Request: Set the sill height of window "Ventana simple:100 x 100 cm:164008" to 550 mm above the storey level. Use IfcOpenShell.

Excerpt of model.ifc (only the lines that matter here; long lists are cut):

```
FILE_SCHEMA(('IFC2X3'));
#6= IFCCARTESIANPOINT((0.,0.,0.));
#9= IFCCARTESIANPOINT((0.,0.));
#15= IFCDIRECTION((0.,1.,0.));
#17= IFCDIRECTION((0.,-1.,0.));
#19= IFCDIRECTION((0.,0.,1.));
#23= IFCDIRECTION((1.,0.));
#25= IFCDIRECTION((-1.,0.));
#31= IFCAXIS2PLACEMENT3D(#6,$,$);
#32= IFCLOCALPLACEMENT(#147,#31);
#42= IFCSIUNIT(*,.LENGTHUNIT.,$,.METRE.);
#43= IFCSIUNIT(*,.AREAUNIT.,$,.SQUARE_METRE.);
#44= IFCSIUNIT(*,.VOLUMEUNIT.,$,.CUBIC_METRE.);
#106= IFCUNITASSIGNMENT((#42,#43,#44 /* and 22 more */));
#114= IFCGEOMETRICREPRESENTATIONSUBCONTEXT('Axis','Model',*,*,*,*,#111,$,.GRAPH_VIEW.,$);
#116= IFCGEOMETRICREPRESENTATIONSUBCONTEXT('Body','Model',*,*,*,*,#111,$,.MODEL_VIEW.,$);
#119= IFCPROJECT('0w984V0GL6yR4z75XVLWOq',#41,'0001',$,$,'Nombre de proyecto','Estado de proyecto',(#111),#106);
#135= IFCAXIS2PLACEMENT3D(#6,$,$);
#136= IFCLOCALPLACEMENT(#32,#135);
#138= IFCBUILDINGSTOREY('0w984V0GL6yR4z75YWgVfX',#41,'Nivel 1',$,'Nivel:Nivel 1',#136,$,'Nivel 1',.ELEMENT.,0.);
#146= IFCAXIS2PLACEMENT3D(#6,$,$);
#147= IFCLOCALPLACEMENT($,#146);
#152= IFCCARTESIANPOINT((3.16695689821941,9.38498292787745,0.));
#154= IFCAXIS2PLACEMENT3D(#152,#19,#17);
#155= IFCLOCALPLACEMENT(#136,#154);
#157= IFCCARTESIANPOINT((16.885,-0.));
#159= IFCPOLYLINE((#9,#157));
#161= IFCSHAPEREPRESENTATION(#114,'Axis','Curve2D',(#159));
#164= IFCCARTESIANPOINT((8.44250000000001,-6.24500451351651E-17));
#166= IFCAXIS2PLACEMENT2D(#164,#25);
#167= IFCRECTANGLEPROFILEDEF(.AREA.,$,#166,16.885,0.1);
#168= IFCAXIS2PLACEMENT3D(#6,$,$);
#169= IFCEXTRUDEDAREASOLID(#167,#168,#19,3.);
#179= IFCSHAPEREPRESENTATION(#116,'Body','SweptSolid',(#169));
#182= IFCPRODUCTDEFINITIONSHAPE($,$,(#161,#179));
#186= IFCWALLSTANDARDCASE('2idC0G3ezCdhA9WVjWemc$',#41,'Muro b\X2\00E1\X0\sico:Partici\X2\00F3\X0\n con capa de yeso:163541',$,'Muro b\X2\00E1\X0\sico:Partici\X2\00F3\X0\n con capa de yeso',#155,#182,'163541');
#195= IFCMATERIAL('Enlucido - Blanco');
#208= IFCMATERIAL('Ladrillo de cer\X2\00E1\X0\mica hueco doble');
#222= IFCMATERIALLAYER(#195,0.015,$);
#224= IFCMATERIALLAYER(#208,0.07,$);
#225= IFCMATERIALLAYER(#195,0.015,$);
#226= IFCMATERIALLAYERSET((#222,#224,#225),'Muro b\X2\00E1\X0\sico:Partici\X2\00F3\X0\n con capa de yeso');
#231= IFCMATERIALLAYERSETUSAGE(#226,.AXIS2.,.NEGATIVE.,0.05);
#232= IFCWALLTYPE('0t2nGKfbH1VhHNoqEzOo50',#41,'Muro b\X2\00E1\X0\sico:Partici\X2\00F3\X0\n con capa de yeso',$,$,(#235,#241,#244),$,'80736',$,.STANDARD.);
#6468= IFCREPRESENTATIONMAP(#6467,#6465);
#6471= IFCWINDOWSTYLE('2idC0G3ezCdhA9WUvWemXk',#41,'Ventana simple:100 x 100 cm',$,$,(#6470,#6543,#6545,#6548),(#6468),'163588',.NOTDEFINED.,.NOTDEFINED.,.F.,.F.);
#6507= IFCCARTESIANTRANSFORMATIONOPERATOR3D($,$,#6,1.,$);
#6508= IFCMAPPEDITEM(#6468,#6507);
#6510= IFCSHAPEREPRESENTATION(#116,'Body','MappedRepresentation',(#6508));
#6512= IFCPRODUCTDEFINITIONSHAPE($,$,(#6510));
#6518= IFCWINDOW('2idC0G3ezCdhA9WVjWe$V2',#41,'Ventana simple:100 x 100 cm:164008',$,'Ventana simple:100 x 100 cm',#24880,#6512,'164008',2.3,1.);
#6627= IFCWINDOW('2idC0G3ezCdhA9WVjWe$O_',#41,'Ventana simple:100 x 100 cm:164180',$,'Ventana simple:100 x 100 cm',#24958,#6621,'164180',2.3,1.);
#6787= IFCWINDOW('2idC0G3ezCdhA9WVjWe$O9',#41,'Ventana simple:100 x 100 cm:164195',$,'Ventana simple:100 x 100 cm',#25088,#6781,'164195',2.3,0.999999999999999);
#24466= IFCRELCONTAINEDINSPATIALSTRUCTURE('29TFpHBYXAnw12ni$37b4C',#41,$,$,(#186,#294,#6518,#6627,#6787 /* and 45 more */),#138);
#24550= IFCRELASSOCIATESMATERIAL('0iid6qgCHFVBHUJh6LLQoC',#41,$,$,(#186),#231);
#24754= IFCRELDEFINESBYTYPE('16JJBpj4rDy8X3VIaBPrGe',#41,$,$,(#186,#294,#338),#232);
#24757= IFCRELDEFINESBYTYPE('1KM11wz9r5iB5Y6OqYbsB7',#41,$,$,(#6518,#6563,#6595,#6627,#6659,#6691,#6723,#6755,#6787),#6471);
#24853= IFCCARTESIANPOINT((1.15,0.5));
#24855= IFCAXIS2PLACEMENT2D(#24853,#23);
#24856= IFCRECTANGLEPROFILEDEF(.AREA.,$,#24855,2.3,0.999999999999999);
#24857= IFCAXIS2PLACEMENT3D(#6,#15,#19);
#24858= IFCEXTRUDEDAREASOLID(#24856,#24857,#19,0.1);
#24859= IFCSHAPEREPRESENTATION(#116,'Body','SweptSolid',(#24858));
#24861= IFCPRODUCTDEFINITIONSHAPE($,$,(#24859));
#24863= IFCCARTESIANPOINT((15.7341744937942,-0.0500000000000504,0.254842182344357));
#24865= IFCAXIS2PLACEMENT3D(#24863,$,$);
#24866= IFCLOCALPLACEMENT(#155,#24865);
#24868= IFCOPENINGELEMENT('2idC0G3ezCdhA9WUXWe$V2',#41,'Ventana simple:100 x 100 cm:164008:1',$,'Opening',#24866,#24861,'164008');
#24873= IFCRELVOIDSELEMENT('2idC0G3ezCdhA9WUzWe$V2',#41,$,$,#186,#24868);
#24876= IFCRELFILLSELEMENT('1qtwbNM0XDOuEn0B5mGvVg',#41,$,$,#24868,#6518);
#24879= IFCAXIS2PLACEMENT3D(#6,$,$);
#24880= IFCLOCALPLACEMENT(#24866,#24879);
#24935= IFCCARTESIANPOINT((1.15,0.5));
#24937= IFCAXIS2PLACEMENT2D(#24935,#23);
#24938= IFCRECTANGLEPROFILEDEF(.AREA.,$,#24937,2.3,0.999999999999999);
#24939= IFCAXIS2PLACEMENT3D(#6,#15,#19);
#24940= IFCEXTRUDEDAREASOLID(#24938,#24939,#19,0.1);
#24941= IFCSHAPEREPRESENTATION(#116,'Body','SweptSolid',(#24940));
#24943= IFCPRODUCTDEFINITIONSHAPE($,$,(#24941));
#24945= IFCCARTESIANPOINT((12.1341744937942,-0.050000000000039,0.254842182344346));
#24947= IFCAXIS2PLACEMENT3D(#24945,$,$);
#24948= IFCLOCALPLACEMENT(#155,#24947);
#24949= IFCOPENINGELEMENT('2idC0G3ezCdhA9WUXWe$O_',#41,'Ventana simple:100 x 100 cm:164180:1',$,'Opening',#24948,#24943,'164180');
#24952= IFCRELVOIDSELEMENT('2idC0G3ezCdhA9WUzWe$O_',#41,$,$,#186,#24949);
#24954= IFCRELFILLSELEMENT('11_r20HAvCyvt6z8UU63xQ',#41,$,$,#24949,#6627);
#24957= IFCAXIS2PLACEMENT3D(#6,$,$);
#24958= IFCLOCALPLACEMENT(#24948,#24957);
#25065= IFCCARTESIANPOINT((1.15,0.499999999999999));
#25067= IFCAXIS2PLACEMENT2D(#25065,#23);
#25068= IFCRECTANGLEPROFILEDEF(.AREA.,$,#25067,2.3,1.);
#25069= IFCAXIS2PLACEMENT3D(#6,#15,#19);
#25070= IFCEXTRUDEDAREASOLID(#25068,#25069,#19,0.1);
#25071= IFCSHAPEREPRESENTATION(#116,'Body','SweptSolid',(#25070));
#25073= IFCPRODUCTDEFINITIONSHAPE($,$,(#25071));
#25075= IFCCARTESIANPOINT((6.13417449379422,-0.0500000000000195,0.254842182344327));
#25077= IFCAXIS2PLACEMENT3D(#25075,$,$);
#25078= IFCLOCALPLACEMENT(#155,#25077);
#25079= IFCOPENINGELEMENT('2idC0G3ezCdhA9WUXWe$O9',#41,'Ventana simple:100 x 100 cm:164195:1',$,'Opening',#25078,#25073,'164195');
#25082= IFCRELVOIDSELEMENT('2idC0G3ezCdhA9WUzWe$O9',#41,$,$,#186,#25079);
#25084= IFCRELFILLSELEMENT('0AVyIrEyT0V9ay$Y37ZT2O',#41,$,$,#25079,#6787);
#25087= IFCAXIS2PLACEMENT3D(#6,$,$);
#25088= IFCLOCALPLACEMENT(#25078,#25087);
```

```python
import numpy as np
import ifcopenshell
import ifcopenshell.api.geometry
import ifcopenshell.geom
import ifcopenshell.util.element
import ifcopenshell.util.placement
import ifcopenshell.util.shape
import ifcopenshell.util.unit

model = ifcopenshell.open("model.ifc")
unit_scale = ifcopenshell.util.unit.calculate_unit_scale(model)

window = model.by_guid("2idC0G3ezCdhA9WVjWe$V2")
opening = window.FillsVoids[0].RelatingOpeningElement
storey = ifcopenshell.util.element.get_container(window, ifc_class="IfcBuildingStorey")
level = ifcopenshell.util.placement.get_local_placement(storey.ObjectPlacement)[2, 3]

# The opening's origin need not be at the sill, so measure its lowest point.
shape = ifcopenshell.geom.create_shape(ifcopenshell.geom.settings(), opening)
bottom = ifcopenshell.util.shape.get_shape_bottom_elevation(shape, shape.geometry) / unit_scale
dz = level + 0.55 - bottom

shift = np.array([0.0, 0.0, dz])
# The window is placed relative to its opening, so it follows when the opening moves.
matrix = ifcopenshell.util.placement.get_local_placement(opening.ObjectPlacement)
matrix[:3, 3] += shift
ifcopenshell.api.geometry.edit_object_placement(
    model, product=opening, matrix=matrix, is_si=False, should_transform_children=True
)

print(f"moved by {dz * unit_scale:+.3f} m")

model.write("model_edited.ifc")
```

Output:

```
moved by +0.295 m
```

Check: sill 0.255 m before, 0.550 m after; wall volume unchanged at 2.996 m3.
